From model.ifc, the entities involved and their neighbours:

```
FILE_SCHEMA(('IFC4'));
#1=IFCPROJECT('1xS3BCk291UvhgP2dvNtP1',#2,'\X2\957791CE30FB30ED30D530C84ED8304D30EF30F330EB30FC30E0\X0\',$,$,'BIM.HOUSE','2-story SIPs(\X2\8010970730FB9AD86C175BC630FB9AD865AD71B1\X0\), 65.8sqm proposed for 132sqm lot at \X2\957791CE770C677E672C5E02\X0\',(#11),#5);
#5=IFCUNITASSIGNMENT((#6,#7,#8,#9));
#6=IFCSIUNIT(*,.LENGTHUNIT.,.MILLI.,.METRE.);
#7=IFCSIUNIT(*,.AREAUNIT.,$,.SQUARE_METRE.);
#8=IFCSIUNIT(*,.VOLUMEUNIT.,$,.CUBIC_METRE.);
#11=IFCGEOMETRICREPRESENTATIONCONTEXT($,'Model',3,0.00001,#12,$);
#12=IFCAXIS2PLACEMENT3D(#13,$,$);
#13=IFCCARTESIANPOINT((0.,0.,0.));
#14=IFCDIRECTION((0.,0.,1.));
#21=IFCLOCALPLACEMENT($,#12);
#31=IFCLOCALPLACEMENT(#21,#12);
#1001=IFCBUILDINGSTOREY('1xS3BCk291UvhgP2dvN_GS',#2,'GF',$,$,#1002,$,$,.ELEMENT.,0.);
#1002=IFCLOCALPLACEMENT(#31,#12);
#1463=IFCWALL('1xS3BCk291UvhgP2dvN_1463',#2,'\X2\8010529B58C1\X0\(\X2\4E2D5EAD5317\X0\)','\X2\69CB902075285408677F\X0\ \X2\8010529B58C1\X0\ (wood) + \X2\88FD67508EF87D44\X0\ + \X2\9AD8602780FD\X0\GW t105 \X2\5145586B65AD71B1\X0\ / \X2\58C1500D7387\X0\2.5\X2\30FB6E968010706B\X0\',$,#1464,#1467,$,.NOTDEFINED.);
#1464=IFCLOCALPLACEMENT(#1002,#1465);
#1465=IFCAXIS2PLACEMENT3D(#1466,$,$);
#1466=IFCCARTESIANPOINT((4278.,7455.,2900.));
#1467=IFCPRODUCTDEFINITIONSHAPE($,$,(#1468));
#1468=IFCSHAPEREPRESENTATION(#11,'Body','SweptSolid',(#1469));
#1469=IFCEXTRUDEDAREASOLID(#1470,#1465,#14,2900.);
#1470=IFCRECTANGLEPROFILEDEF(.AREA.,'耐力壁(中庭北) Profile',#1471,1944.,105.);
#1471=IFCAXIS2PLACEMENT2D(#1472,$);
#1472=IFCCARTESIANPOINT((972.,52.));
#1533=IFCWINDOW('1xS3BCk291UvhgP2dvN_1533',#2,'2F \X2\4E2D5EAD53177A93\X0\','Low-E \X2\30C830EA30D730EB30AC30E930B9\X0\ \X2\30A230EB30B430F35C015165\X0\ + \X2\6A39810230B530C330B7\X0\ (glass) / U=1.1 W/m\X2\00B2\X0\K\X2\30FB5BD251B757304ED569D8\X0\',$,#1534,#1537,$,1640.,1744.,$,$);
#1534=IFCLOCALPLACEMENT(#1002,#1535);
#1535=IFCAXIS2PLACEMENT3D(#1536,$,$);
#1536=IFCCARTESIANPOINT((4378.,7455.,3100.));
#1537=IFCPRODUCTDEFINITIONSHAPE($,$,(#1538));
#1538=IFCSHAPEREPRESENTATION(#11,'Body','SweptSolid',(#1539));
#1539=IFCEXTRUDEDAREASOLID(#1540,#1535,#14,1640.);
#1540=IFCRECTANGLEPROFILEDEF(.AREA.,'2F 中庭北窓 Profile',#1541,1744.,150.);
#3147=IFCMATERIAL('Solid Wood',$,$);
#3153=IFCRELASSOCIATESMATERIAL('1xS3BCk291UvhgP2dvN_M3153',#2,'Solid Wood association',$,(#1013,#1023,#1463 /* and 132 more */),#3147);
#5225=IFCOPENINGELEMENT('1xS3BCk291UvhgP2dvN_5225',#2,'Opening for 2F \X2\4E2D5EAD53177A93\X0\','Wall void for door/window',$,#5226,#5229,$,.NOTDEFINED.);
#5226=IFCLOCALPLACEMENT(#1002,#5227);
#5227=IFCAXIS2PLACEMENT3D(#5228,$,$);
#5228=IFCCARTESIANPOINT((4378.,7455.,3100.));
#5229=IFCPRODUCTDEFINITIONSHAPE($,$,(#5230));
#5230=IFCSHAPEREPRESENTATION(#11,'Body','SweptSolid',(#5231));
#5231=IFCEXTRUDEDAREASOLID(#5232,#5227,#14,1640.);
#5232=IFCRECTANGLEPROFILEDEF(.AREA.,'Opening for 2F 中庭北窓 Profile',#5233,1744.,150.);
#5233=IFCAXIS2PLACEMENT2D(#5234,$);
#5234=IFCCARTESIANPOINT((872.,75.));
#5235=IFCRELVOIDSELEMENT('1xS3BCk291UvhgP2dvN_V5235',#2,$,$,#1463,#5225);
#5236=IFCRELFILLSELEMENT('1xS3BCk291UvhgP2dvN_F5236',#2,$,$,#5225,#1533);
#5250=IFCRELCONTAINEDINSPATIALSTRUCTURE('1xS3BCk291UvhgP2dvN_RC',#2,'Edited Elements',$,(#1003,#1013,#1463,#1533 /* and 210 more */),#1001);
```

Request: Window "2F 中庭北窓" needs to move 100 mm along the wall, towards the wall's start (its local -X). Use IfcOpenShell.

```python
import ifcopenshell
import ifcopenshell.api.geometry
import ifcopenshell.util.placement
import ifcopenshell.util.unit

model = ifcopenshell.open("model.ifc")
unit_scale = ifcopenshell.util.unit.calculate_unit_scale(model)

window = model.by_id(1533)
opening = window.FillsVoids[0].RelatingOpeningElement
wall = opening.VoidsElements[0].RelatingBuildingElement

wall_matrix = ifcopenshell.util.placement.get_local_placement(wall.ObjectPlacement)
shift = wall_matrix[:3, 0] * -0.1 / unit_scale
before = ifcopenshell.util.placement.get_local_placement(window.ObjectPlacement)[:3, 3].copy()

# The window is not placed relative to its opening, so move both.
for product in (opening, window):
    matrix = ifcopenshell.util.placement.get_local_placement(product.ObjectPlacement)
    matrix[:3, 3] += shift
    ifcopenshell.api.geometry.edit_object_placement(model, product=product, matrix=matrix, is_si=False)

after = ifcopenshell.util.placement.get_local_placement(window.ObjectPlacement)[:3, 3]
print("window moved by", (after - before).round(3) + 0.0)

model.write("model_v2.ifc")
```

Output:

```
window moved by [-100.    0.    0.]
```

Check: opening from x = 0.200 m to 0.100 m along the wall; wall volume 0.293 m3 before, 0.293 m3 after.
